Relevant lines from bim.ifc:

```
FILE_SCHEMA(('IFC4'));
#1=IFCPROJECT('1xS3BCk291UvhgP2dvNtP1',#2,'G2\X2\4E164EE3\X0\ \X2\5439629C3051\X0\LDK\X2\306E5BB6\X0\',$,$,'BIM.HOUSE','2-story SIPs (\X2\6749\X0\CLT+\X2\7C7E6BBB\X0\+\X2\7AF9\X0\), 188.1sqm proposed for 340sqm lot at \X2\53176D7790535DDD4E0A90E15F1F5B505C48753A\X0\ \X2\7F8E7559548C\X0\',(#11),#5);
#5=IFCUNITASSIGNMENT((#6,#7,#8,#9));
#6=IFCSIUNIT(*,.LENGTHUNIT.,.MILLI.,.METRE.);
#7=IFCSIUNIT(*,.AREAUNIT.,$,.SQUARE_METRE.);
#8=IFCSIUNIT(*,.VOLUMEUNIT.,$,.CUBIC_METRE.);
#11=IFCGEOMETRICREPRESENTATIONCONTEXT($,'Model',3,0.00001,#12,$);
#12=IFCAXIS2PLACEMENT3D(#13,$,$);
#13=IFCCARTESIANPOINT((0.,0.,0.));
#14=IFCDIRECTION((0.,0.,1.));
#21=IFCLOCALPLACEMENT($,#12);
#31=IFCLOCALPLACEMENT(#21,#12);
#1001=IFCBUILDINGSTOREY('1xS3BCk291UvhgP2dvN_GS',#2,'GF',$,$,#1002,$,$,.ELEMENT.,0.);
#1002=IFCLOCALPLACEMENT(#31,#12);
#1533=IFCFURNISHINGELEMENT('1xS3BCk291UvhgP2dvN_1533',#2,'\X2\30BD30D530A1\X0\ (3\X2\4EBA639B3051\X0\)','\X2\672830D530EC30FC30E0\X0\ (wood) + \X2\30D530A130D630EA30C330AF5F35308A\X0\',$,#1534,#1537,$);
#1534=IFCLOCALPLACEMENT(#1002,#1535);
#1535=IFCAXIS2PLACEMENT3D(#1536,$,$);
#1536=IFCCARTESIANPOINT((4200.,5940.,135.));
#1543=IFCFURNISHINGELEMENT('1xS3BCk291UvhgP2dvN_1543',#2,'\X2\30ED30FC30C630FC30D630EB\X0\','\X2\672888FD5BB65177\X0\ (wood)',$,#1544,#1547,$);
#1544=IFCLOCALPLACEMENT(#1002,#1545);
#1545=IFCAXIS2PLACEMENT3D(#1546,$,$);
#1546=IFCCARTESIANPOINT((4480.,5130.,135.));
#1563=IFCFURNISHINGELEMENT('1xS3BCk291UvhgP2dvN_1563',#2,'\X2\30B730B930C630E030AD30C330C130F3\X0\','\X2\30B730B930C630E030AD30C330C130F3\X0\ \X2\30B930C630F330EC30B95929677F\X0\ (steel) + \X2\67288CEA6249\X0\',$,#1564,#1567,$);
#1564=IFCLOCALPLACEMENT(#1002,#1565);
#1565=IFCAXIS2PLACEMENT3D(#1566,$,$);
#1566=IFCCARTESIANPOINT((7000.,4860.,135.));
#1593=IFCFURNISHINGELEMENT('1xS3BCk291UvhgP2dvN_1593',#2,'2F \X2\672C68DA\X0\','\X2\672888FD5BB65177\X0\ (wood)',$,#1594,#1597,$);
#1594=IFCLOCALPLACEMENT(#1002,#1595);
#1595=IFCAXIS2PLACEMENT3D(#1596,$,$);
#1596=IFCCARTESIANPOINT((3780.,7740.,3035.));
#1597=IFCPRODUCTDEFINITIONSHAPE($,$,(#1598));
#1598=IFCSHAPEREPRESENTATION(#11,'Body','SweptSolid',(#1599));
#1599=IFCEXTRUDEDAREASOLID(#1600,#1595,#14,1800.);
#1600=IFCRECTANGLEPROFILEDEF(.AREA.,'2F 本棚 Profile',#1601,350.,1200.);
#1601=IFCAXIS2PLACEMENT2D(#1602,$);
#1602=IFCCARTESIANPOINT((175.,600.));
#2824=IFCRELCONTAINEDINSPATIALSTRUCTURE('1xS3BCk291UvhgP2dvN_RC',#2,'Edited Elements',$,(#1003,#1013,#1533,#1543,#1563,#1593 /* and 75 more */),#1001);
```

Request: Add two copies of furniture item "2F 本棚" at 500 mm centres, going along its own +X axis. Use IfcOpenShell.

```python
import ifcopenshell
import ifcopenshell.api.geometry
import ifcopenshell.api.root
import ifcopenshell.util.element
import ifcopenshell.util.placement
import ifcopenshell.util.unit

model = ifcopenshell.open("bim.ifc")
unit_scale = ifcopenshell.util.unit.calculate_unit_scale(model)


def reuse_history(source, copy):
    """copy_class also copies each property set's owner history, people and application; keep the originals."""
    for rel in copy.IsDefinedBy:
        if rel.is_a("IfcRelDefinesByProperties") and (history := rel.RelatingPropertyDefinition.OwnerHistory):
            rel.RelatingPropertyDefinition.OwnerHistory = source.OwnerHistory
            ifcopenshell.util.element.remove_deep2(model, history)


source = model.by_guid("1xS3BCk291UvhgP2dvN_1593")
base = ifcopenshell.util.placement.get_local_placement(source.ObjectPlacement)
step = base[:3, 0] * 0.5 / unit_scale

for i in range(1, 3):
    copy = ifcopenshell.api.root.copy_class(model, product=source)
    copy.Representation = ifcopenshell.util.element.copy_deep(
        model, source.Representation, exclude=["IfcGeometricRepresentationContext", "IfcRepresentationMap"]
    )
    reuse_history(source, copy)
    matrix = base.copy()
    matrix[:3, 3] += i * step
    print("added at", matrix[:3, 3].round(3) + 0.0)
    ifcopenshell.api.geometry.edit_object_placement(model, product=copy, matrix=matrix, is_si=False)

model.write("bim_rev.ifc")
```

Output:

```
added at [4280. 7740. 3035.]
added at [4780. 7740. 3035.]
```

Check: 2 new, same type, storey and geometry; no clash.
